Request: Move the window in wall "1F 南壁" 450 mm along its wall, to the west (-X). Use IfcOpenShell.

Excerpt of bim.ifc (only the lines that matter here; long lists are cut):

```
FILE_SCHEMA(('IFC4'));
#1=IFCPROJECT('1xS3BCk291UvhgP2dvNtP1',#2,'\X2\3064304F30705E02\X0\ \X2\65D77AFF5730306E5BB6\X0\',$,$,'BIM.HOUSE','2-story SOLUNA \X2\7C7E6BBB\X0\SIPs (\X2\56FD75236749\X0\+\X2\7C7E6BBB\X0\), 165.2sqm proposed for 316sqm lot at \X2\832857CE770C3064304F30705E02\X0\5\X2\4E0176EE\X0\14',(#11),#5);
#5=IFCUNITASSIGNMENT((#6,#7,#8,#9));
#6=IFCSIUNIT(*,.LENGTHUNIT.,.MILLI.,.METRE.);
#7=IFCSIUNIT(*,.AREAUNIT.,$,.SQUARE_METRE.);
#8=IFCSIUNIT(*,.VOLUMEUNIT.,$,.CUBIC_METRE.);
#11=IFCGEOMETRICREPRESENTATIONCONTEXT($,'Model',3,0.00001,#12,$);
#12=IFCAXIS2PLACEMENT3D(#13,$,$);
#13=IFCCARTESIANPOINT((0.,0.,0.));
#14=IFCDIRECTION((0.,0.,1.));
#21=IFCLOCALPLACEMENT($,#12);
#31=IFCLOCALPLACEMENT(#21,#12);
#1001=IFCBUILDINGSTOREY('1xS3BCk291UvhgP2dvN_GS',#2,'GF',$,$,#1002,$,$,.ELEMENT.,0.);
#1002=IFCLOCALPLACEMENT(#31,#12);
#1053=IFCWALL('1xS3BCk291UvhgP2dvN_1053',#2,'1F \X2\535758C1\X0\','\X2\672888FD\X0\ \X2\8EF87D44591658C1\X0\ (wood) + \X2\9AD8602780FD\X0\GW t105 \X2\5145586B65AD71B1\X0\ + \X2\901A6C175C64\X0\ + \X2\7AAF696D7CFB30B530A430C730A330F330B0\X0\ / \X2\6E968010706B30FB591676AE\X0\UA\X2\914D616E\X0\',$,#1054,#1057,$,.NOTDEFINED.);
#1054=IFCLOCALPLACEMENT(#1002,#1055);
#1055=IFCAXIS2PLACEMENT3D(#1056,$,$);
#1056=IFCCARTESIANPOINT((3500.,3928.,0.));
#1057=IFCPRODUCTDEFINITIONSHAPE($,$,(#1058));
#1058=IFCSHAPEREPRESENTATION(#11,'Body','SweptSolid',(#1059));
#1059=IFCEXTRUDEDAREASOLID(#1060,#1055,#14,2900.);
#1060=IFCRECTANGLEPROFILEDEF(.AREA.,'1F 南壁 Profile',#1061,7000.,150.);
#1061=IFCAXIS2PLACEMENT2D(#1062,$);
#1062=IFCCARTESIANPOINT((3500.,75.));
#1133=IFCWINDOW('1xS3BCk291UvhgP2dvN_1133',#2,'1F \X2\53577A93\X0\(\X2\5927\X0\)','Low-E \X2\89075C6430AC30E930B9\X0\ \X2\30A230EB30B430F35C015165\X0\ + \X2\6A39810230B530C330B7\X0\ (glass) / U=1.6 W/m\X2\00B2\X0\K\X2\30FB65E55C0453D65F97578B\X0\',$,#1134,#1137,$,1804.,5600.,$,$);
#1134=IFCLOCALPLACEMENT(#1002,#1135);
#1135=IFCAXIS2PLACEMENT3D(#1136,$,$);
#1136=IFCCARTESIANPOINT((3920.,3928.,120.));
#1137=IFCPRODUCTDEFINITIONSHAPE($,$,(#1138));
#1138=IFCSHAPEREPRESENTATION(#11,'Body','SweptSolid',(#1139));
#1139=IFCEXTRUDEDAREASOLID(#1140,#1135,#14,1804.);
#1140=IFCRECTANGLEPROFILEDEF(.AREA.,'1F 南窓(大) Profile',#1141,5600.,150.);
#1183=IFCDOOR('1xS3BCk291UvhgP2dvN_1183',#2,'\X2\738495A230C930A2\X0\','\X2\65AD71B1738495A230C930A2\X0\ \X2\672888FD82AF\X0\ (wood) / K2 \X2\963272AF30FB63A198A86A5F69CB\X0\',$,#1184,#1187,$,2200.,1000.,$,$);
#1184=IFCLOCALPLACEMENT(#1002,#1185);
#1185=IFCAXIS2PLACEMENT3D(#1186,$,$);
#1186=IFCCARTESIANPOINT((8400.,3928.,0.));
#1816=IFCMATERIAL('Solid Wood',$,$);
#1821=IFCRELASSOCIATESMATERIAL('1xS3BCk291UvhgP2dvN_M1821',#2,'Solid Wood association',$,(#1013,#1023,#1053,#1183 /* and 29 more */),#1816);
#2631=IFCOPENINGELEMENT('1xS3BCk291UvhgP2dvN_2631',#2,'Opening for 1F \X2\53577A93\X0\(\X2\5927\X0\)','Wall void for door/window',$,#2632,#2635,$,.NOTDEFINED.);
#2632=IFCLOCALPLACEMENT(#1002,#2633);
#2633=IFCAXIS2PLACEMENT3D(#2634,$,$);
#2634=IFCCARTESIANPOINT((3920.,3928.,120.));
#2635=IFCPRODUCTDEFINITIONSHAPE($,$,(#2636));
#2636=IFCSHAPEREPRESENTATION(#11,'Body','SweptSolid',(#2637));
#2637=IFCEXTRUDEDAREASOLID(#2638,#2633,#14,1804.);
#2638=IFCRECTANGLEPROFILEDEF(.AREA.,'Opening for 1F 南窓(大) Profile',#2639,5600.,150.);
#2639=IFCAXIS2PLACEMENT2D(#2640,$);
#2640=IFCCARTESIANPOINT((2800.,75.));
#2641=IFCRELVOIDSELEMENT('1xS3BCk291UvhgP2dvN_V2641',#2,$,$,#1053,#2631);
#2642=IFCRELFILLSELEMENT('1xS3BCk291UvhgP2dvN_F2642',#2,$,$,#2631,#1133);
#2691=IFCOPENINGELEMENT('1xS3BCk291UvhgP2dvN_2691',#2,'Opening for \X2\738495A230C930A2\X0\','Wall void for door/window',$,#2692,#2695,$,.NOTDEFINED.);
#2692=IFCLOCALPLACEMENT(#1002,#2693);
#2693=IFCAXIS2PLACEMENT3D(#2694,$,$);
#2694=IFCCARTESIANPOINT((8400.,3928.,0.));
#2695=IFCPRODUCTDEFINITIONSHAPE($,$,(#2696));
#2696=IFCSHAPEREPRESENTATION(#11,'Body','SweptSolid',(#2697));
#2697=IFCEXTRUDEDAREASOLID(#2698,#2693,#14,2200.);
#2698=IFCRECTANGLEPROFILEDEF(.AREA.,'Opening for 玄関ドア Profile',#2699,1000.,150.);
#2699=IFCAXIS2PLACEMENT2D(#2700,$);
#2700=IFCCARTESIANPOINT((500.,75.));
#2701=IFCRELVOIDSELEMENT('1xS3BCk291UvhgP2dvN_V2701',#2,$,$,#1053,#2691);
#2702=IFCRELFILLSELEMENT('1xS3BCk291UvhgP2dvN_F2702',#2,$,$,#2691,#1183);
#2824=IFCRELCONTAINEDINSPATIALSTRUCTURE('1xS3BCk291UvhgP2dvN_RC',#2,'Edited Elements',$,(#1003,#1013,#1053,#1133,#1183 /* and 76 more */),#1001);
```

```python
import ifcopenshell
import ifcopenshell.api.geometry
import ifcopenshell.util.placement
import ifcopenshell.util.unit

model = ifcopenshell.open("bim.ifc")
unit_scale = ifcopenshell.util.unit.calculate_unit_scale(model)

window = model.by_guid("1xS3BCk291UvhgP2dvN_1133")
opening = window.FillsVoids[0].RelatingOpeningElement
wall = opening.VoidsElements[0].RelatingBuildingElement

wall_matrix = ifcopenshell.util.placement.get_local_placement(wall.ObjectPlacement)
shift = wall_matrix[:3, 0] * -0.45 / unit_scale
before = ifcopenshell.util.placement.get_local_placement(window.ObjectPlacement)[:3, 3].copy()

# The window is not placed relative to its opening, so move both.
for product in (opening, window):
    matrix = ifcopenshell.util.placement.get_local_placement(product.ObjectPlacement)
    matrix[:3, 3] += shift
    ifcopenshell.api.geometry.edit_object_placement(model, product=product, matrix=matrix, is_si=False)

after = ifcopenshell.util.placement.get_local_placement(window.ObjectPlacement)[:3, 3]
print("window moved by", (after - before).round(3) + 0.0)

model.write("bim_edited.ifc")
```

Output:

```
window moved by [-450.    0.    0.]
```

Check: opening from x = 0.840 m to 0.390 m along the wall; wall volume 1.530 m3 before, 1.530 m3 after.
